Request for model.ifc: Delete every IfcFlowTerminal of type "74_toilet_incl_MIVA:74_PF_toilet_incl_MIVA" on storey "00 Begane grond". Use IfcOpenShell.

First a look at what the model holds.

```python
import ifcopenshell
import ifcopenshell.util.element

model = ifcopenshell.open("model.ifc")
print(model.schema)
storey = next(s for s in model.by_type("IfcBuildingStorey") if s.Name == "00 Begane grond")
terminals = [e for e in ifcopenshell.util.element.get_decomposition(storey) if e.is_a("IfcFlowTerminal")]
seen = {}
for e in terminals:
    element_type = ifcopenshell.util.element.get_type(e)
    name = element_type.Name if element_type not in (None, e) else None
    seen[name] = seen.get(name, 0) + 1
for name, count in sorted(seen.items(), key=str):
    print(count, "x", name)
```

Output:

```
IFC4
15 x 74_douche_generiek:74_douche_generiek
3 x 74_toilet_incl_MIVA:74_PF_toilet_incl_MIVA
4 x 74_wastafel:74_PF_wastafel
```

```python
import ifcopenshell
import ifcopenshell.api.root
import ifcopenshell.util.element

model = ifcopenshell.open("model.ifc")

storey = next(s for s in model.by_type("IfcBuildingStorey") if s.Name == "00 Begane grond")
terminals = [e for e in ifcopenshell.util.element.get_decomposition(storey) if e.is_a("IfcFlowTerminal")]
targets = [e for e in terminals if (t := ifcopenshell.util.element.get_type(e)) not in (None, e) and t.Name == "74_toilet_incl_MIVA:74_PF_toilet_incl_MIVA"]

for e in targets:
    ifcopenshell.api.root.remove_product(model, product=e)
print(len(targets), "removed")

model.write("model_rev.ifc")
```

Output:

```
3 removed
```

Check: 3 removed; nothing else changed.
